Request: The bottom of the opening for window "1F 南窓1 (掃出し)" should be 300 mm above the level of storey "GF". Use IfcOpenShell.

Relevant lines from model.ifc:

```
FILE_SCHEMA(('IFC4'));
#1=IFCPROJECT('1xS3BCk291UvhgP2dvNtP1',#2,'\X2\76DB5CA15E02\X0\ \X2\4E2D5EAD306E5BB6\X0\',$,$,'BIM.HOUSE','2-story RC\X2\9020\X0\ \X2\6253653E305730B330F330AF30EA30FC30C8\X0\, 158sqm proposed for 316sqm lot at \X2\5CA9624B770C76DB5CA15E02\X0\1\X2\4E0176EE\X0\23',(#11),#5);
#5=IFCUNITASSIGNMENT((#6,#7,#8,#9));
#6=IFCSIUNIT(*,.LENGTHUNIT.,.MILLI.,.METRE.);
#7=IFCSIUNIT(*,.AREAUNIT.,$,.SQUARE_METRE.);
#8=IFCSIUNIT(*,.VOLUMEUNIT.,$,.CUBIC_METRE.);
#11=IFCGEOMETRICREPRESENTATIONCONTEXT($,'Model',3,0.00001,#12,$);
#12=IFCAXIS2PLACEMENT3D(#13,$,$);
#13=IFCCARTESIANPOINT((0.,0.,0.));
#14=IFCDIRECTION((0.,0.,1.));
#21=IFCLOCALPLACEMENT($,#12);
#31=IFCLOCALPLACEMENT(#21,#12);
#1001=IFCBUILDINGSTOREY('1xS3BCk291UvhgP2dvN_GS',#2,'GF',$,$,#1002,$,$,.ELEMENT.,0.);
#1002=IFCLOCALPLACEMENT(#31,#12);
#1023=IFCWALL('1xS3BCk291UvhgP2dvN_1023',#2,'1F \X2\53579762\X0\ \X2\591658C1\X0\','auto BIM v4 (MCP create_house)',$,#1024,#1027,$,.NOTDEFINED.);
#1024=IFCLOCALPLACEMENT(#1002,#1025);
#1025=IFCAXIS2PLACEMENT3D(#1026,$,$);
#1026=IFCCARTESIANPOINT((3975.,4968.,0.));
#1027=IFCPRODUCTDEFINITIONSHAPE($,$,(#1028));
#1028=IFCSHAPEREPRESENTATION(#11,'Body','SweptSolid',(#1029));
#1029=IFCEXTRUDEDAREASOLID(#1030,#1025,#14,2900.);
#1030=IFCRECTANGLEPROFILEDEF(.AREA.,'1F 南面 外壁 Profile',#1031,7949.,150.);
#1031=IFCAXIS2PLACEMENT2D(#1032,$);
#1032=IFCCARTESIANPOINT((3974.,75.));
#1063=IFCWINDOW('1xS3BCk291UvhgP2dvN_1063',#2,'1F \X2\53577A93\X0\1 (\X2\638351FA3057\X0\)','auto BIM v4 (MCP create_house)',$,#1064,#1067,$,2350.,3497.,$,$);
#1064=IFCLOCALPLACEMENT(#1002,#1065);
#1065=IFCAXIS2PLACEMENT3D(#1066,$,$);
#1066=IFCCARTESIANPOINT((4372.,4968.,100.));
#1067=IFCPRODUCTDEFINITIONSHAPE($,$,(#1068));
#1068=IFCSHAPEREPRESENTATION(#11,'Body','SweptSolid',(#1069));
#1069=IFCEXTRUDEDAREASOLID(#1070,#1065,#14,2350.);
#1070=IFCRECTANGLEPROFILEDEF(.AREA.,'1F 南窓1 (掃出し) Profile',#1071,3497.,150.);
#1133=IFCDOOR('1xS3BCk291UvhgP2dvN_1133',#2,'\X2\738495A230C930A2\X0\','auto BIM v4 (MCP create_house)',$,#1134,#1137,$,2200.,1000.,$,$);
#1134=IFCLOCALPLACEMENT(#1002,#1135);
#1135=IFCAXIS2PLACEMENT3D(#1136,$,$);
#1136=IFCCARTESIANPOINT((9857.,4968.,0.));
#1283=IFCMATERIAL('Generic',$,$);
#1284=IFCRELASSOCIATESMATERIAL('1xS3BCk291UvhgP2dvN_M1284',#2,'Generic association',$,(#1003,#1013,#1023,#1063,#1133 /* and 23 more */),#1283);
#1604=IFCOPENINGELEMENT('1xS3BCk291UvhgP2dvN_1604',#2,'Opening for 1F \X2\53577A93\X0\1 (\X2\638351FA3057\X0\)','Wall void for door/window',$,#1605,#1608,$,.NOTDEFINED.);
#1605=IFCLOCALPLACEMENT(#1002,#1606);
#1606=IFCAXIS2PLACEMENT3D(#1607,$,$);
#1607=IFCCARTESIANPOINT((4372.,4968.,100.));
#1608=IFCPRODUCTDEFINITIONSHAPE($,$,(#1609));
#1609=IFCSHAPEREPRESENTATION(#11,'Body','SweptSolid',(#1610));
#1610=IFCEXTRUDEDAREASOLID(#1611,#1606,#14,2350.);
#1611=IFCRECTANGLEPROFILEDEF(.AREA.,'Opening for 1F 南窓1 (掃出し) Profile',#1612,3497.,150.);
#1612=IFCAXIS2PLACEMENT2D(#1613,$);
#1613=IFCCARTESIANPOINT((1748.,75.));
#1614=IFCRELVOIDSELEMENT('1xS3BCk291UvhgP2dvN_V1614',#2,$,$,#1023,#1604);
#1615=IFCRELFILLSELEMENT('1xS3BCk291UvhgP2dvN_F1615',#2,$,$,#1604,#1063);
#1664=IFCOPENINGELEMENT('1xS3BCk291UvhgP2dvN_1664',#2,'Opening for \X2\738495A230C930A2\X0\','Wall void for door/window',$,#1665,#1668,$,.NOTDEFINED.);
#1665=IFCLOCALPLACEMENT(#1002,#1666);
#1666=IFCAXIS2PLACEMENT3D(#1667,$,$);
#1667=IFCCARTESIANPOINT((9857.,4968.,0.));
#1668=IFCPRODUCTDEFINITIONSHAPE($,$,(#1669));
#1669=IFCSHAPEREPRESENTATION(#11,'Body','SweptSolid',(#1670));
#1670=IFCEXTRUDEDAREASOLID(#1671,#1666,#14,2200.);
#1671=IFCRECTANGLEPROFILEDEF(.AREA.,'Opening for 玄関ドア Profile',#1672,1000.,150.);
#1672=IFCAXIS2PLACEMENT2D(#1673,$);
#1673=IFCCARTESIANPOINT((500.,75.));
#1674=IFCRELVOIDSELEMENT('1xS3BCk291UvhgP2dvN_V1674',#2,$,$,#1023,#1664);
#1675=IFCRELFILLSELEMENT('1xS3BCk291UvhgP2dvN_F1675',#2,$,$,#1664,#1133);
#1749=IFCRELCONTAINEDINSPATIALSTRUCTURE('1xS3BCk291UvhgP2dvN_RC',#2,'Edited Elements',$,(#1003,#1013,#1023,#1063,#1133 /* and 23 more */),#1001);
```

```python
import numpy as np
import ifcopenshell
import ifcopenshell.api.geometry
import ifcopenshell.geom
import ifcopenshell.util.element
import ifcopenshell.util.placement
import ifcopenshell.util.shape
import ifcopenshell.util.unit

model = ifcopenshell.open("model.ifc")
unit_scale = ifcopenshell.util.unit.calculate_unit_scale(model)

window = model.by_guid("1xS3BCk291UvhgP2dvN_1063")
opening = window.FillsVoids[0].RelatingOpeningElement
storey = ifcopenshell.util.element.get_container(window, ifc_class="IfcBuildingStorey")
level = ifcopenshell.util.placement.get_local_placement(storey.ObjectPlacement)[2, 3]

# The opening's origin need not be at the sill, so measure its lowest point.
shape = ifcopenshell.geom.create_shape(ifcopenshell.geom.settings(), opening)
bottom = ifcopenshell.util.shape.get_shape_bottom_elevation(shape, shape.geometry) / unit_scale
dz = level + 0.3 / unit_scale - bottom

shift = np.array([0.0, 0.0, dz])
# The window is not placed relative to its opening, so move both.
for product in (opening, window):
    matrix = ifcopenshell.util.placement.get_local_placement(product.ObjectPlacement)
    matrix[:3, 3] += shift
    ifcopenshell.api.geometry.edit_object_placement(model, product=product, matrix=matrix, is_si=False)

print(f"moved by {dz * unit_scale:+.3f} m")

model.write("model_edited.ifc")
```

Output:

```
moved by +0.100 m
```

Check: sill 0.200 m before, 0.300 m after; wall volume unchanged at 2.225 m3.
